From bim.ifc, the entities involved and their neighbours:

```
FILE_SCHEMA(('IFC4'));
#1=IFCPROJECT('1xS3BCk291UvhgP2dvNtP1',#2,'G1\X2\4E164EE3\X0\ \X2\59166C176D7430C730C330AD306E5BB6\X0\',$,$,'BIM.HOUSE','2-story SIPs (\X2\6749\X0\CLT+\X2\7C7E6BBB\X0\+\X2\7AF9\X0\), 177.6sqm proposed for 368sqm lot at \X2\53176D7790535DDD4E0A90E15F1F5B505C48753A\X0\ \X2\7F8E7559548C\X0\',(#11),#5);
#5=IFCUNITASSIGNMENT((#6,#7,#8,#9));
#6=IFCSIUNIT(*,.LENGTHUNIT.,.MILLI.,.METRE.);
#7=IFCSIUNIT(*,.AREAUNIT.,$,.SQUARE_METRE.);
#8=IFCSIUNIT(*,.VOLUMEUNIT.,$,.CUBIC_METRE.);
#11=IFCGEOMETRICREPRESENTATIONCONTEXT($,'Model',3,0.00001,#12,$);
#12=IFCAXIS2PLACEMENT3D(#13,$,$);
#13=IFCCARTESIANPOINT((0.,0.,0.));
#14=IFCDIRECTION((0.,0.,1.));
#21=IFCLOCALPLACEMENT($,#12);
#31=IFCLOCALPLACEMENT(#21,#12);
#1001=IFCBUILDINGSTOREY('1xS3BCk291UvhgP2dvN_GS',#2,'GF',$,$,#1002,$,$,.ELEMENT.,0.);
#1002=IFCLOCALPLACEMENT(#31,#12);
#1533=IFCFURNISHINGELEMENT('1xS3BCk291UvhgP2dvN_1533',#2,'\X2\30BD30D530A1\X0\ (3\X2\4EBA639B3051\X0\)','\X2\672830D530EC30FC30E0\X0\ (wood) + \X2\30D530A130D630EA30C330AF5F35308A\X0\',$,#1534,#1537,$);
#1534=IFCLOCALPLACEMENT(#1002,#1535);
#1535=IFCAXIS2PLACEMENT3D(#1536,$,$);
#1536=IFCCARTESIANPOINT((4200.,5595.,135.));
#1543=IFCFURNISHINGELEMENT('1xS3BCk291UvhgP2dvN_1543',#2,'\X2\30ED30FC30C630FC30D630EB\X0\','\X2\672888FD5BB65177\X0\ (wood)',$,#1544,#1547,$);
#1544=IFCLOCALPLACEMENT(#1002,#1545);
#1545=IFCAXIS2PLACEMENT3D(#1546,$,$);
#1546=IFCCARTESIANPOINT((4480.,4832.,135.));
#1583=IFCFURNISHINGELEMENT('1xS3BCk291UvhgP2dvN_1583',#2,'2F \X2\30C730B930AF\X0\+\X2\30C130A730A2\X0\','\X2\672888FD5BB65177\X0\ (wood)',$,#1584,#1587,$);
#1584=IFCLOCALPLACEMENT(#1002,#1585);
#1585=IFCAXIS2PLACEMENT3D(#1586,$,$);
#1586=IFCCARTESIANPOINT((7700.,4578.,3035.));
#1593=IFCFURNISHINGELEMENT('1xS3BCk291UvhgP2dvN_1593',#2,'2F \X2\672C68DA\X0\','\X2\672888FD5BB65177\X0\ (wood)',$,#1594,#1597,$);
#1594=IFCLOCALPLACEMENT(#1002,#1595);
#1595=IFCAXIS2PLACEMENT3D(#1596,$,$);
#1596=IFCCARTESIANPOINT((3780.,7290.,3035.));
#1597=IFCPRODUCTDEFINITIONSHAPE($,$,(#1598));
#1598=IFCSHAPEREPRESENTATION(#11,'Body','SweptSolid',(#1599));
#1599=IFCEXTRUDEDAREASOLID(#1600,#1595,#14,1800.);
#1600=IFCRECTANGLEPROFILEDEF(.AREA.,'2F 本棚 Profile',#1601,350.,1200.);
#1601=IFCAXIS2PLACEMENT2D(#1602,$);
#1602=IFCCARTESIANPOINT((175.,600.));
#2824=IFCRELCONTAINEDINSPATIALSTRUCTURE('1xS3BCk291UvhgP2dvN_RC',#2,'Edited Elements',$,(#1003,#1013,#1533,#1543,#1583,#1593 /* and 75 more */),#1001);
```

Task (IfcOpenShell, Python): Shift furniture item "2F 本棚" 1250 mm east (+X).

```python
import ifcopenshell
import ifcopenshell.api.geometry
import ifcopenshell.util.placement

model = ifcopenshell.open("bim.ifc")

item = model.by_guid("1xS3BCk291UvhgP2dvN_1593")
matrix = ifcopenshell.util.placement.get_local_placement(item.ObjectPlacement)
matrix[0, 3] += 1250.0
ifcopenshell.api.geometry.edit_object_placement(model, product=item, matrix=matrix, is_si=False)

print(ifcopenshell.util.placement.get_local_placement(item.ObjectPlacement).round(3) + 0.0)

model.write("bim_edited.ifc")
```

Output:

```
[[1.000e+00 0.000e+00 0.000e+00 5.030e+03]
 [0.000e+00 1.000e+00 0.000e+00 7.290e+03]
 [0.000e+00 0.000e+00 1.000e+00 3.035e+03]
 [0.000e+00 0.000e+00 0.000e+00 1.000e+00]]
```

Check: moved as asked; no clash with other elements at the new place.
